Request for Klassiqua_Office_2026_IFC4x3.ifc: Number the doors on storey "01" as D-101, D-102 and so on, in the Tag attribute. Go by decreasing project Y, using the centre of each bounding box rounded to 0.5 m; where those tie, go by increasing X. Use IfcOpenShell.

First a look at what the model holds.

```python
import ifcopenshell
import ifcopenshell.util.element
import ifcopenshell.util.placement

model = ifcopenshell.open("Klassiqua_Office_2026_IFC4x3.ifc")
print(model.schema)
storey = next(s for s in model.by_type("IfcBuildingStorey") if s.Name == "01")
doors = [e for e in ifcopenshell.util.element.get_decomposition(storey) if e.is_a("IfcDoor")]
for e in sorted(doors, key=lambda e: e.id()):
    origin = ifcopenshell.util.placement.get_local_placement(e.ObjectPlacement)[:3, 3]
    print(e.id(), e.Tag, e.Name, origin.round(2) + 0.0, sep=" | ")
```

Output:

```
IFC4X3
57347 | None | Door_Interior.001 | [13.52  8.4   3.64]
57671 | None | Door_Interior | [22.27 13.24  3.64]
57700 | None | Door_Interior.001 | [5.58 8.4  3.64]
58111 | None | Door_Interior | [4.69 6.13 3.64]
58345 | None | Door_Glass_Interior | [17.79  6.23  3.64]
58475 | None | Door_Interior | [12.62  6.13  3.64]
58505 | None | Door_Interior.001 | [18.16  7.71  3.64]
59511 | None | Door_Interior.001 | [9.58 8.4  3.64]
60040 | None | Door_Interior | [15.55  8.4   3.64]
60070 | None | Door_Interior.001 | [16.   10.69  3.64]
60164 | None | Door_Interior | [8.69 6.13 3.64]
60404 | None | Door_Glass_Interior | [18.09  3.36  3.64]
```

```python
import ifcopenshell
import ifcopenshell.geom
import ifcopenshell.util.element
import ifcopenshell.util.shape

model = ifcopenshell.open("Klassiqua_Office_2026_IFC4x3.ifc")
settings = ifcopenshell.geom.settings()
settings.set("use-world-coords", True)


def centre(element):
    shape = ifcopenshell.geom.create_shape(settings, element)
    return ifcopenshell.util.shape.get_bbox_centroid(shape.geometry)


storey = next(s for s in model.by_type("IfcBuildingStorey") if s.Name == "01")
doors = [e for e in ifcopenshell.util.element.get_decomposition(storey) if e.is_a("IfcDoor")]

# Insertion points can sit at a corner or the storey origin, so sort by the geometry (in metres).
centres = {e: centre(e) for e in doors}
doors.sort(key=lambda e: (-round(centres[e][1] / 0.5), centres[e][0]))

for i, e in enumerate(doors, start=1):
    number = f"D-1{i:02d}"
    e.Tag = number
    print(e.id(), number)

model.write("Klassiqua_Office_2026_IFC4x3_updated.ifc")
```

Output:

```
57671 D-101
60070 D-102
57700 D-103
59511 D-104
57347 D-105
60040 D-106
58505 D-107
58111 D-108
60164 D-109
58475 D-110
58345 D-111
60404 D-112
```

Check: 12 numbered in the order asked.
